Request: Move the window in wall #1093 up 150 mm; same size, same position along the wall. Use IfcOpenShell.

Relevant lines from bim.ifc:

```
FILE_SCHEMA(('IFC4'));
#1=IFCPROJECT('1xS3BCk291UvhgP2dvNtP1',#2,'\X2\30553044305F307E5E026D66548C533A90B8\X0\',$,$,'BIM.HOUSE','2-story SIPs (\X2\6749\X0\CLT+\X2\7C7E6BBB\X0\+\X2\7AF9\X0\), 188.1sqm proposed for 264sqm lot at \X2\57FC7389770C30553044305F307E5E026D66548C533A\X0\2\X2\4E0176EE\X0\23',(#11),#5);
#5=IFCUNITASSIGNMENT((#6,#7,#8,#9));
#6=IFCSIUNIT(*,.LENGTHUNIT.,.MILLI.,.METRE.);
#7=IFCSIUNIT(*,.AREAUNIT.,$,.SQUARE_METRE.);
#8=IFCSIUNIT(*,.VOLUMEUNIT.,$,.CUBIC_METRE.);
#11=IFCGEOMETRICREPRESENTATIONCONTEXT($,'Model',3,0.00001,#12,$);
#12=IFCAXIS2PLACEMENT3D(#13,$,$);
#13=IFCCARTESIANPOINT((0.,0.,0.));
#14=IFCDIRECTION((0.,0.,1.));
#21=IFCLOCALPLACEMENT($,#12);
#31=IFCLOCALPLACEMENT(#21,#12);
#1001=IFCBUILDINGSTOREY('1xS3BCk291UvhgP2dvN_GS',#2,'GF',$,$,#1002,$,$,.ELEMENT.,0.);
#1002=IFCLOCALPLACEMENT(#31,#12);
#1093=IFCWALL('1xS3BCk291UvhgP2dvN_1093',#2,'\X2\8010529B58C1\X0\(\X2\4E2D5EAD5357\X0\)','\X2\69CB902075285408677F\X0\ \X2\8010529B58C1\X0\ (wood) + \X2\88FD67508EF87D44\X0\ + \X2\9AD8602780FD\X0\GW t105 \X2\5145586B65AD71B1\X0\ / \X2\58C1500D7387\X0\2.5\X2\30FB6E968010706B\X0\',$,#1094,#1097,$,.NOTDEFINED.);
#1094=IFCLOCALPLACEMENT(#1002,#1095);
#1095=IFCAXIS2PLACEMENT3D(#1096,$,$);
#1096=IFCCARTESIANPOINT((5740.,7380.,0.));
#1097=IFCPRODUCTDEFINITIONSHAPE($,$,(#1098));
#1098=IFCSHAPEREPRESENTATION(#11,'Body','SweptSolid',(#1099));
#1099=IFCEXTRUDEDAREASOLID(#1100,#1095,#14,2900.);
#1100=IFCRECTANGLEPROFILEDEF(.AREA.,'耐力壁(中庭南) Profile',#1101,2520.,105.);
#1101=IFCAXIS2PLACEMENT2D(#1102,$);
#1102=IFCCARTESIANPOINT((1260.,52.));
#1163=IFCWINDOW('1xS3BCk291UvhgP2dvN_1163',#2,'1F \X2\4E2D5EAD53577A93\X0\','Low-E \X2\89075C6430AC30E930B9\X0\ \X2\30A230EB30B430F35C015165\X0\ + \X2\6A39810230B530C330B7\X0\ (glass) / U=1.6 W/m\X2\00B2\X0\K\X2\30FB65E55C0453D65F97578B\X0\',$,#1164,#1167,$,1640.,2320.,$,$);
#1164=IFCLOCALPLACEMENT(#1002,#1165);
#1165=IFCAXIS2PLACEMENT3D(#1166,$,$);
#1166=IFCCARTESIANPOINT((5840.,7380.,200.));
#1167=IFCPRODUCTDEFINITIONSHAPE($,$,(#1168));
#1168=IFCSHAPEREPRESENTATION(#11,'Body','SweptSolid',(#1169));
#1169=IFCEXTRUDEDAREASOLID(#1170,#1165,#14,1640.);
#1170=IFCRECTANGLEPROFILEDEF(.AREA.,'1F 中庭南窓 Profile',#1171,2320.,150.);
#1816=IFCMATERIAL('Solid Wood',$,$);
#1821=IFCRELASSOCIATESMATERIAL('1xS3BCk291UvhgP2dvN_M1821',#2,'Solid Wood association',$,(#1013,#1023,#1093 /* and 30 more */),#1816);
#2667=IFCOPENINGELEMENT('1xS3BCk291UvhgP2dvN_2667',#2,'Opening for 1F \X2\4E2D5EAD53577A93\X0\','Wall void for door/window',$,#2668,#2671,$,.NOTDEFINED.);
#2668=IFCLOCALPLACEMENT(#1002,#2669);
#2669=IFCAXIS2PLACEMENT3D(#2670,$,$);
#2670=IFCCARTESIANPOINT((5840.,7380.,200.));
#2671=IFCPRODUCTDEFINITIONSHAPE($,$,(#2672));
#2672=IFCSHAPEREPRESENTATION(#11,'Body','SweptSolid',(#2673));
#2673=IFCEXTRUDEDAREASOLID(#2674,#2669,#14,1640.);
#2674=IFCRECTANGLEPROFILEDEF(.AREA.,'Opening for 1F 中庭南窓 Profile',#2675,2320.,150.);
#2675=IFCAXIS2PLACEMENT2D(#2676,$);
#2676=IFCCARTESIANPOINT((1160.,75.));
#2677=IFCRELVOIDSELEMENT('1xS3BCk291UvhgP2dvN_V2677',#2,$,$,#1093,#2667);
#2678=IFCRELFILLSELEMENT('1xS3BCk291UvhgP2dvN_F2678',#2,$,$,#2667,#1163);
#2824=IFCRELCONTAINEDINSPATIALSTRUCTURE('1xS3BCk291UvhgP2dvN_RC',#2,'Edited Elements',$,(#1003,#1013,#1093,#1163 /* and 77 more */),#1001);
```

```python
import numpy as np
import ifcopenshell
import ifcopenshell.api.geometry
import ifcopenshell.util.placement
import ifcopenshell.util.unit

model = ifcopenshell.open("bim.ifc")
unit_scale = ifcopenshell.util.unit.calculate_unit_scale(model)

window = model.by_guid("1xS3BCk291UvhgP2dvN_1163")
opening = window.FillsVoids[0].RelatingOpeningElement
dz = 0.15 / unit_scale

shift = np.array([0.0, 0.0, dz])
# The window is not placed relative to its opening, so move both.
for product in (opening, window):
    matrix = ifcopenshell.util.placement.get_local_placement(product.ObjectPlacement)
    matrix[:3, 3] += shift
    ifcopenshell.api.geometry.edit_object_placement(model, product=product, matrix=matrix, is_si=False)

print(f"moved by {dz * unit_scale:+.3f} m")

model.write("bim-out.ifc")
```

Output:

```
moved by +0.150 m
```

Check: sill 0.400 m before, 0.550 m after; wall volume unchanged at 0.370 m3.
